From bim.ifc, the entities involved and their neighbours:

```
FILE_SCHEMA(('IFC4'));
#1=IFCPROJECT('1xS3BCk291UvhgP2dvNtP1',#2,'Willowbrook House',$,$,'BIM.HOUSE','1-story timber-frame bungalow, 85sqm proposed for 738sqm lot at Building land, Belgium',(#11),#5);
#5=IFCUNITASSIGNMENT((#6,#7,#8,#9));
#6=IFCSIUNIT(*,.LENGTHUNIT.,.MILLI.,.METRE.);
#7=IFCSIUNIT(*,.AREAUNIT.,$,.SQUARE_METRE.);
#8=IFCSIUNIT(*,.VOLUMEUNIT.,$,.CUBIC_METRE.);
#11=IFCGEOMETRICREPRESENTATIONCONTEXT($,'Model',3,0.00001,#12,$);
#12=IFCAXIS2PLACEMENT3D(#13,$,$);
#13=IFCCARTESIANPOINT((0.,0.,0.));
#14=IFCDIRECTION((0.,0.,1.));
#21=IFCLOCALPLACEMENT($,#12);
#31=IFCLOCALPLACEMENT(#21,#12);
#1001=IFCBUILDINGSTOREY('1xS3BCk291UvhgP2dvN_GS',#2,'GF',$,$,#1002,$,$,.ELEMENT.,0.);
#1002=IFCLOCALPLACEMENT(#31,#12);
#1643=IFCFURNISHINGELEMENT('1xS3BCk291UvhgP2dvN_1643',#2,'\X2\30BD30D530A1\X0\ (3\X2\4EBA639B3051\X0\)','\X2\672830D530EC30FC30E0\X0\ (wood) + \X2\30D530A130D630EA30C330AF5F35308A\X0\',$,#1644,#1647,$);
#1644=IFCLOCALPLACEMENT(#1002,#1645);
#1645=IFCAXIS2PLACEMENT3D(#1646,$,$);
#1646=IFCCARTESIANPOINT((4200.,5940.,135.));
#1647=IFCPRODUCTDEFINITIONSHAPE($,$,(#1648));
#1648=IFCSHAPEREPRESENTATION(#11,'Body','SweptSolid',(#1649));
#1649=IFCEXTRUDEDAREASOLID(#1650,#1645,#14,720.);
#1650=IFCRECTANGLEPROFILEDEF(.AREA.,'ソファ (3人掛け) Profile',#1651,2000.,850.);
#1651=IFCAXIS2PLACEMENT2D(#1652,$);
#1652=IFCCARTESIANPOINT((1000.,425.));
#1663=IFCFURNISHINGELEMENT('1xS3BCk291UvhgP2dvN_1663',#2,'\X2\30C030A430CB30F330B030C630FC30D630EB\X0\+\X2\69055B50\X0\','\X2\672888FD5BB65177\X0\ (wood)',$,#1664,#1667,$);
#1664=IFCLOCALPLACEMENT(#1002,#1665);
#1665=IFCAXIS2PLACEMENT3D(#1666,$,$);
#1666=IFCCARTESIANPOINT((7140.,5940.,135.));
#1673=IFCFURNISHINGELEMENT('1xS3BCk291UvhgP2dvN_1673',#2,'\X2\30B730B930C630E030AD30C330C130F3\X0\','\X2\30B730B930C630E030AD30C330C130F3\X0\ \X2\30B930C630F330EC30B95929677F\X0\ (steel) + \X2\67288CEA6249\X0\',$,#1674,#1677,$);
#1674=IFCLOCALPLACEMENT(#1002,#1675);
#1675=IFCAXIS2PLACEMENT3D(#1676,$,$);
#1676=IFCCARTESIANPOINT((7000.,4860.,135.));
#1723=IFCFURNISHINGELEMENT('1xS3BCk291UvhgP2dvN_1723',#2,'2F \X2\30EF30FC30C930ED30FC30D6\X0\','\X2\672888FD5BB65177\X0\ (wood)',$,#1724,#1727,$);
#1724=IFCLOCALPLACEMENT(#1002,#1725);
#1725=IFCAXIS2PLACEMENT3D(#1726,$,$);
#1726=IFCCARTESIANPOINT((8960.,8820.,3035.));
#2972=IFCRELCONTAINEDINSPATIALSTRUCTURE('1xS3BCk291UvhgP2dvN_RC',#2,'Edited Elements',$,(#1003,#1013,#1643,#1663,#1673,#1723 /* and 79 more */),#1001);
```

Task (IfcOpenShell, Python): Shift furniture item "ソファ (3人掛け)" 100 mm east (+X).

```python
import ifcopenshell
import ifcopenshell.api.geometry
import ifcopenshell.util.placement
import ifcopenshell.util.unit

model = ifcopenshell.open("bim.ifc")
unit_scale = ifcopenshell.util.unit.calculate_unit_scale(model)

item = model.by_guid("1xS3BCk291UvhgP2dvN_1643")
matrix = ifcopenshell.util.placement.get_local_placement(item.ObjectPlacement)
matrix[0, 3] += 0.1 / unit_scale
ifcopenshell.api.geometry.edit_object_placement(model, product=item, matrix=matrix, is_si=False)

print(ifcopenshell.util.placement.get_local_placement(item.ObjectPlacement).round(3) + 0.0)

model.write("bim-out.ifc")
```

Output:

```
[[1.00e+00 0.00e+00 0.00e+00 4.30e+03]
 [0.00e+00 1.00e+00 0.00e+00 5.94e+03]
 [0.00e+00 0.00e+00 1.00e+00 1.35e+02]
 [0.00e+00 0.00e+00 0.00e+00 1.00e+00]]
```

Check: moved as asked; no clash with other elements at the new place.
